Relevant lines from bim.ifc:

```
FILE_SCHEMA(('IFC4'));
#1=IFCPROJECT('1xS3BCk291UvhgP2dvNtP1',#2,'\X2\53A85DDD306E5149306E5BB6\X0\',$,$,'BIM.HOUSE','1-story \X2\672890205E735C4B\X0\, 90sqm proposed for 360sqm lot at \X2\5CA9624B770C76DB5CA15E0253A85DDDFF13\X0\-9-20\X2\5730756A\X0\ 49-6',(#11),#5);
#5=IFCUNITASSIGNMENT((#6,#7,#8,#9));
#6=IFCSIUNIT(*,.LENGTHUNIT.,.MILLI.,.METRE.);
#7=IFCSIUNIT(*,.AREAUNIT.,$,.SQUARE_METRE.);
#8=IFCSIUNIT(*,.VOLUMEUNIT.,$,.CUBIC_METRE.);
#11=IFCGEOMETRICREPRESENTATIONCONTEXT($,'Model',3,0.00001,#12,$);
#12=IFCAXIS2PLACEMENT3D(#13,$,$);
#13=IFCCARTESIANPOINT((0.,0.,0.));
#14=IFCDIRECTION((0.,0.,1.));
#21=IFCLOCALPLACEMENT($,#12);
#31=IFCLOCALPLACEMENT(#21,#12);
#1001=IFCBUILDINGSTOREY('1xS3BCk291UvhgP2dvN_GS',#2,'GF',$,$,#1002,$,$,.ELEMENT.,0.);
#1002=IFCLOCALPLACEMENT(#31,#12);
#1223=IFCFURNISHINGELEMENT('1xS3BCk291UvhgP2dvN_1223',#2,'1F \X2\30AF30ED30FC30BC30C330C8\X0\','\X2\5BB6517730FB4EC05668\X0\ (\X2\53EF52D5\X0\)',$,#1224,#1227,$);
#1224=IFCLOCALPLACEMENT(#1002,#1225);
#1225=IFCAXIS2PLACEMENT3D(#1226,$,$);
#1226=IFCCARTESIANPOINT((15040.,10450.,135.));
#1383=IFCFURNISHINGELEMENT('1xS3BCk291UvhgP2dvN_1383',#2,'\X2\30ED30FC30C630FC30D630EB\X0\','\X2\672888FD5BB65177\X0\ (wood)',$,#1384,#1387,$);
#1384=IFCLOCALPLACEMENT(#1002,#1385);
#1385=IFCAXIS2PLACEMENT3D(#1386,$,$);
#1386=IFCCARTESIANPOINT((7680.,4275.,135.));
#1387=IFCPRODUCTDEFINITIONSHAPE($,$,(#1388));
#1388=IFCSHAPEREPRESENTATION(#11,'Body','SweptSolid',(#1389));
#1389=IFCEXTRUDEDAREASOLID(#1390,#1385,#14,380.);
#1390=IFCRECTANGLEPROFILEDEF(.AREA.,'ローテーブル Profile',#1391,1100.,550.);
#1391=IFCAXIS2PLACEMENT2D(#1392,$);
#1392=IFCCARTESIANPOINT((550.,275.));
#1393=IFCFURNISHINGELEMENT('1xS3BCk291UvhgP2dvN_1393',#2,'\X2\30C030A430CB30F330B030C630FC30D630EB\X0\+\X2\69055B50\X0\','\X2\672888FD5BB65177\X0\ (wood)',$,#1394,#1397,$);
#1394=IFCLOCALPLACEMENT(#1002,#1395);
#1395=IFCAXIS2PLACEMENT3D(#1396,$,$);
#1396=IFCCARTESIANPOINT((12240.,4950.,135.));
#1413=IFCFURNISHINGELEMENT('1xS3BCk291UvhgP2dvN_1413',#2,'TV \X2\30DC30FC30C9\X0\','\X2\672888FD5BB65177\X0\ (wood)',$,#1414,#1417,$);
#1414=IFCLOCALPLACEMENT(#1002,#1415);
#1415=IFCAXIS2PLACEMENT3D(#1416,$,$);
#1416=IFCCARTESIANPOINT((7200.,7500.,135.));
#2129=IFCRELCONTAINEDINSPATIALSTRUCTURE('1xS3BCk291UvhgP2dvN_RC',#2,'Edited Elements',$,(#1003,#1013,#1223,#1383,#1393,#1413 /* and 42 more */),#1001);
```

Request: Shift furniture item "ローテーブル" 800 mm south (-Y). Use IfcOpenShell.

```python
import ifcopenshell
import ifcopenshell.api.geometry
import ifcopenshell.util.placement
import ifcopenshell.util.unit

model = ifcopenshell.open("bim.ifc")
unit_scale = ifcopenshell.util.unit.calculate_unit_scale(model)

item = model.by_guid("1xS3BCk291UvhgP2dvN_1383")
matrix = ifcopenshell.util.placement.get_local_placement(item.ObjectPlacement)
matrix[1, 3] -= 0.8 / unit_scale
ifcopenshell.api.geometry.edit_object_placement(model, product=item, matrix=matrix, is_si=False)

print(ifcopenshell.util.placement.get_local_placement(item.ObjectPlacement).round(3) + 0.0)

model.write("bim_updated.ifc")
```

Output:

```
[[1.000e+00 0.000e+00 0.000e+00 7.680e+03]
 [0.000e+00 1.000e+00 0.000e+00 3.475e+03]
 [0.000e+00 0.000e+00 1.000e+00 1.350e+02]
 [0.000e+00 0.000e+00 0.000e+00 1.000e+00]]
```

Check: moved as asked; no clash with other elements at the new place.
